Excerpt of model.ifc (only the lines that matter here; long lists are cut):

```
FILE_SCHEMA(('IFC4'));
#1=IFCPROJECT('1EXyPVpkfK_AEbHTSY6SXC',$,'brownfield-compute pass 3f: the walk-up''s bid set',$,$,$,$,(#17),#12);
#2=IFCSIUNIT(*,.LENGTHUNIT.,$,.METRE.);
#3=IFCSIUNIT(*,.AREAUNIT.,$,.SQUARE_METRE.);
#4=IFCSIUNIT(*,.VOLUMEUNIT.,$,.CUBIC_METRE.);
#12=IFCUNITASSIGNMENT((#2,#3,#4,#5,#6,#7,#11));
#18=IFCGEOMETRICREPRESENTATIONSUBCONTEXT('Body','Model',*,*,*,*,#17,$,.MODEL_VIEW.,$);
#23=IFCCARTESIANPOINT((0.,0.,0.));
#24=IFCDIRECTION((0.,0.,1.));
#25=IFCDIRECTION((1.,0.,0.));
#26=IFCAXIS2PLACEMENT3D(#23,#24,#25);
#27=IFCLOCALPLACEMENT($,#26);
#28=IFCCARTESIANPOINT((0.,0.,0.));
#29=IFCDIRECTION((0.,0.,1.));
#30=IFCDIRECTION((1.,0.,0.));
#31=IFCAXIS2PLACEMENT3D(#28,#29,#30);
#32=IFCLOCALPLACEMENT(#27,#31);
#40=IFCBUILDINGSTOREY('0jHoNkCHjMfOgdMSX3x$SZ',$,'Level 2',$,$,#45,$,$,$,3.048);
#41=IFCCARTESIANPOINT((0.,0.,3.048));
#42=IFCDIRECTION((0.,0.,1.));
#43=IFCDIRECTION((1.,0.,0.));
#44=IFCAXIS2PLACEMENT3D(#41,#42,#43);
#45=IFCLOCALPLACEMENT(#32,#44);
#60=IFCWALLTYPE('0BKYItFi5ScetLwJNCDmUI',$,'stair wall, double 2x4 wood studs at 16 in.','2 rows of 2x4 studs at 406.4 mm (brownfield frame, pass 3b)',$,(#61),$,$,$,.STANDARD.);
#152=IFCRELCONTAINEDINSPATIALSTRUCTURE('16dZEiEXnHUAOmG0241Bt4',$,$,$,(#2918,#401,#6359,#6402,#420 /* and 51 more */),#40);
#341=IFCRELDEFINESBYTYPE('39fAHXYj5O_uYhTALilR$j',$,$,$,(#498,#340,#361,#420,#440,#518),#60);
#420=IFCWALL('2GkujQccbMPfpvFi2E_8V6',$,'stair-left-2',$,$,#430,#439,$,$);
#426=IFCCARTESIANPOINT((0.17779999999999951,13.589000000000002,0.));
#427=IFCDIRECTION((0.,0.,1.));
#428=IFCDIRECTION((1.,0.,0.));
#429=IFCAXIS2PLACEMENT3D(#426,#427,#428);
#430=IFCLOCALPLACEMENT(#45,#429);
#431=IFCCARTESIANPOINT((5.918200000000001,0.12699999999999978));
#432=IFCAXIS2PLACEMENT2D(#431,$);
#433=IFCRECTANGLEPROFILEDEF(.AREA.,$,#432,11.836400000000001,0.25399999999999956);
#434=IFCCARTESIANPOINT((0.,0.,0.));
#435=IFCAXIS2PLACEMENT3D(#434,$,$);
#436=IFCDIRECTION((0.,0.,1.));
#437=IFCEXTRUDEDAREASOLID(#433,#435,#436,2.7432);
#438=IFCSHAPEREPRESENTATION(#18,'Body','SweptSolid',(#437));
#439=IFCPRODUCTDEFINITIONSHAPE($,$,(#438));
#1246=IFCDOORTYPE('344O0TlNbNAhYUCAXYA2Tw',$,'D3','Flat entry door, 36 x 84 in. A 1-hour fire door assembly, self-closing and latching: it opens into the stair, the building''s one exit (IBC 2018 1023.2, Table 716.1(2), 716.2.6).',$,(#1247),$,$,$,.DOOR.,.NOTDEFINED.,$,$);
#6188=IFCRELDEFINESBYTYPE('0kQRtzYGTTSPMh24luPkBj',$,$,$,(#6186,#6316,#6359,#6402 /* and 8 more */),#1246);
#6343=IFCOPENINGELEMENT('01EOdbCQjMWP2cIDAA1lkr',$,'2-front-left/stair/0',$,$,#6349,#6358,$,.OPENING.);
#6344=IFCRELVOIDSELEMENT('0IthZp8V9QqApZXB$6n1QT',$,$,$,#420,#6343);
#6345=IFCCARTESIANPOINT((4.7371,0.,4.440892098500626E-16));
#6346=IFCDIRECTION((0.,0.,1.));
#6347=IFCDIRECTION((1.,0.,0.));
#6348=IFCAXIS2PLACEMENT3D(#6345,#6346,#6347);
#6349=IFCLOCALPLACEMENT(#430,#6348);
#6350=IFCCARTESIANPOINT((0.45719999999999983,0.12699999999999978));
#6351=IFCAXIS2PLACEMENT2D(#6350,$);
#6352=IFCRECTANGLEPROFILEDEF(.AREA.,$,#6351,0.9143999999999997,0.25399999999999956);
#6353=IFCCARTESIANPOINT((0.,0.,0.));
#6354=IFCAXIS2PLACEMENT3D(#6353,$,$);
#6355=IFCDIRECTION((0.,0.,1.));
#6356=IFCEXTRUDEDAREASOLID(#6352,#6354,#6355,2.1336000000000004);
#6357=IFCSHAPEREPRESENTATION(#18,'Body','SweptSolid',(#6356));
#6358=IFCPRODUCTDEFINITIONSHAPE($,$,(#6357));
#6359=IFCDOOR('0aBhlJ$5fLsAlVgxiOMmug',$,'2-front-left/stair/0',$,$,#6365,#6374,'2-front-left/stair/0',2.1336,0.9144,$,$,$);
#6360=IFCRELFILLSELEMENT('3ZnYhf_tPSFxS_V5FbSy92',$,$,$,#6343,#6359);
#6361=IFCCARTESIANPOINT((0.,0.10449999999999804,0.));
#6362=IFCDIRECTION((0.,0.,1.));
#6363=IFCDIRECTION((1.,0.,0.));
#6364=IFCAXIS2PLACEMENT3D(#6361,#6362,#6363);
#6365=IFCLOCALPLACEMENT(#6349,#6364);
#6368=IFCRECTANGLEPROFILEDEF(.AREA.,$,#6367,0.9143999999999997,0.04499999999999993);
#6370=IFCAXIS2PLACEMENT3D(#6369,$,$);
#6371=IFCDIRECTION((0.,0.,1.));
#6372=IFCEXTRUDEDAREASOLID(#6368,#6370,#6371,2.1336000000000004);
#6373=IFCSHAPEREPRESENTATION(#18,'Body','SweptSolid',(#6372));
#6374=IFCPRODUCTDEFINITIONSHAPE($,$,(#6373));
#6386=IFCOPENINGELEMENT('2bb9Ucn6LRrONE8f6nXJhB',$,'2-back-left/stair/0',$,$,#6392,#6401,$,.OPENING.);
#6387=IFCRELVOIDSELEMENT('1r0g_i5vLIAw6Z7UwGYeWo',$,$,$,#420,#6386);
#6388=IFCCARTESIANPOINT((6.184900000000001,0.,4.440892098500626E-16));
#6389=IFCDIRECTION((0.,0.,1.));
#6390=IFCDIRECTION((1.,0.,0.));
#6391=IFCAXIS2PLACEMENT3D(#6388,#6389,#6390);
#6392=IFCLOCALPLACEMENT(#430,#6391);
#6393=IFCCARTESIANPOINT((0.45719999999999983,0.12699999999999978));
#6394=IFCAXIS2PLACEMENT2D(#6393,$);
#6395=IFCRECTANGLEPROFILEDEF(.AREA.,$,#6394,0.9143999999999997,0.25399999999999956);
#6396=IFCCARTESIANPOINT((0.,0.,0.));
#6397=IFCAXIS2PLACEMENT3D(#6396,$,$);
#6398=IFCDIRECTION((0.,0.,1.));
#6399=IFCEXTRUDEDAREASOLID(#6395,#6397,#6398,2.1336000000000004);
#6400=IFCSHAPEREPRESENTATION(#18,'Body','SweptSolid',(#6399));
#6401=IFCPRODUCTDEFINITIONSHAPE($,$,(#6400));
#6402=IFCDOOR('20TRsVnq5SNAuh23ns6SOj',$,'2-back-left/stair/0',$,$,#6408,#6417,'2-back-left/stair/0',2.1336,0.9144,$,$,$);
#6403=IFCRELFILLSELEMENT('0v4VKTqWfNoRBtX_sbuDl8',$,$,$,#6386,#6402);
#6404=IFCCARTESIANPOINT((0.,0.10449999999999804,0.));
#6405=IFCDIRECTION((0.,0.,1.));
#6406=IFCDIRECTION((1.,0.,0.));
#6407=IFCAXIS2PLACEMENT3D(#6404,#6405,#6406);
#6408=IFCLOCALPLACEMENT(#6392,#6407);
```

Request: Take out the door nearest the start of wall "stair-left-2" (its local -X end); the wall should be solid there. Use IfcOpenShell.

```python
import ifcopenshell
import ifcopenshell.api.feature
import ifcopenshell.api.root
import ifcopenshell.geom
import ifcopenshell.util.shape

model = ifcopenshell.open("model.ifc")
settings = ifcopenshell.geom.settings()


def volume(element):
    """Net volume in cubic metres, openings subtracted."""
    shape = ifcopenshell.geom.create_shape(settings, element)
    return ifcopenshell.util.shape.get_volume(shape.geometry)


door = model.by_guid("0aBhlJ$5fLsAlVgxiOMmug")
opening = door.FillsVoids[0].RelatingOpeningElement
wall = opening.VoidsElements[0].RelatingBuildingElement
before = volume(wall)

ifcopenshell.api.root.remove_product(model, product=door)
ifcopenshell.api.feature.remove_feature(model, feature=opening)

after = volume(wall)

print(f"wall volume {before:.3f} -> {after:.3f} m3")

model.write("model_rev.ifc")
```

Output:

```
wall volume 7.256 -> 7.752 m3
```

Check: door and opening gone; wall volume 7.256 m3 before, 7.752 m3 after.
